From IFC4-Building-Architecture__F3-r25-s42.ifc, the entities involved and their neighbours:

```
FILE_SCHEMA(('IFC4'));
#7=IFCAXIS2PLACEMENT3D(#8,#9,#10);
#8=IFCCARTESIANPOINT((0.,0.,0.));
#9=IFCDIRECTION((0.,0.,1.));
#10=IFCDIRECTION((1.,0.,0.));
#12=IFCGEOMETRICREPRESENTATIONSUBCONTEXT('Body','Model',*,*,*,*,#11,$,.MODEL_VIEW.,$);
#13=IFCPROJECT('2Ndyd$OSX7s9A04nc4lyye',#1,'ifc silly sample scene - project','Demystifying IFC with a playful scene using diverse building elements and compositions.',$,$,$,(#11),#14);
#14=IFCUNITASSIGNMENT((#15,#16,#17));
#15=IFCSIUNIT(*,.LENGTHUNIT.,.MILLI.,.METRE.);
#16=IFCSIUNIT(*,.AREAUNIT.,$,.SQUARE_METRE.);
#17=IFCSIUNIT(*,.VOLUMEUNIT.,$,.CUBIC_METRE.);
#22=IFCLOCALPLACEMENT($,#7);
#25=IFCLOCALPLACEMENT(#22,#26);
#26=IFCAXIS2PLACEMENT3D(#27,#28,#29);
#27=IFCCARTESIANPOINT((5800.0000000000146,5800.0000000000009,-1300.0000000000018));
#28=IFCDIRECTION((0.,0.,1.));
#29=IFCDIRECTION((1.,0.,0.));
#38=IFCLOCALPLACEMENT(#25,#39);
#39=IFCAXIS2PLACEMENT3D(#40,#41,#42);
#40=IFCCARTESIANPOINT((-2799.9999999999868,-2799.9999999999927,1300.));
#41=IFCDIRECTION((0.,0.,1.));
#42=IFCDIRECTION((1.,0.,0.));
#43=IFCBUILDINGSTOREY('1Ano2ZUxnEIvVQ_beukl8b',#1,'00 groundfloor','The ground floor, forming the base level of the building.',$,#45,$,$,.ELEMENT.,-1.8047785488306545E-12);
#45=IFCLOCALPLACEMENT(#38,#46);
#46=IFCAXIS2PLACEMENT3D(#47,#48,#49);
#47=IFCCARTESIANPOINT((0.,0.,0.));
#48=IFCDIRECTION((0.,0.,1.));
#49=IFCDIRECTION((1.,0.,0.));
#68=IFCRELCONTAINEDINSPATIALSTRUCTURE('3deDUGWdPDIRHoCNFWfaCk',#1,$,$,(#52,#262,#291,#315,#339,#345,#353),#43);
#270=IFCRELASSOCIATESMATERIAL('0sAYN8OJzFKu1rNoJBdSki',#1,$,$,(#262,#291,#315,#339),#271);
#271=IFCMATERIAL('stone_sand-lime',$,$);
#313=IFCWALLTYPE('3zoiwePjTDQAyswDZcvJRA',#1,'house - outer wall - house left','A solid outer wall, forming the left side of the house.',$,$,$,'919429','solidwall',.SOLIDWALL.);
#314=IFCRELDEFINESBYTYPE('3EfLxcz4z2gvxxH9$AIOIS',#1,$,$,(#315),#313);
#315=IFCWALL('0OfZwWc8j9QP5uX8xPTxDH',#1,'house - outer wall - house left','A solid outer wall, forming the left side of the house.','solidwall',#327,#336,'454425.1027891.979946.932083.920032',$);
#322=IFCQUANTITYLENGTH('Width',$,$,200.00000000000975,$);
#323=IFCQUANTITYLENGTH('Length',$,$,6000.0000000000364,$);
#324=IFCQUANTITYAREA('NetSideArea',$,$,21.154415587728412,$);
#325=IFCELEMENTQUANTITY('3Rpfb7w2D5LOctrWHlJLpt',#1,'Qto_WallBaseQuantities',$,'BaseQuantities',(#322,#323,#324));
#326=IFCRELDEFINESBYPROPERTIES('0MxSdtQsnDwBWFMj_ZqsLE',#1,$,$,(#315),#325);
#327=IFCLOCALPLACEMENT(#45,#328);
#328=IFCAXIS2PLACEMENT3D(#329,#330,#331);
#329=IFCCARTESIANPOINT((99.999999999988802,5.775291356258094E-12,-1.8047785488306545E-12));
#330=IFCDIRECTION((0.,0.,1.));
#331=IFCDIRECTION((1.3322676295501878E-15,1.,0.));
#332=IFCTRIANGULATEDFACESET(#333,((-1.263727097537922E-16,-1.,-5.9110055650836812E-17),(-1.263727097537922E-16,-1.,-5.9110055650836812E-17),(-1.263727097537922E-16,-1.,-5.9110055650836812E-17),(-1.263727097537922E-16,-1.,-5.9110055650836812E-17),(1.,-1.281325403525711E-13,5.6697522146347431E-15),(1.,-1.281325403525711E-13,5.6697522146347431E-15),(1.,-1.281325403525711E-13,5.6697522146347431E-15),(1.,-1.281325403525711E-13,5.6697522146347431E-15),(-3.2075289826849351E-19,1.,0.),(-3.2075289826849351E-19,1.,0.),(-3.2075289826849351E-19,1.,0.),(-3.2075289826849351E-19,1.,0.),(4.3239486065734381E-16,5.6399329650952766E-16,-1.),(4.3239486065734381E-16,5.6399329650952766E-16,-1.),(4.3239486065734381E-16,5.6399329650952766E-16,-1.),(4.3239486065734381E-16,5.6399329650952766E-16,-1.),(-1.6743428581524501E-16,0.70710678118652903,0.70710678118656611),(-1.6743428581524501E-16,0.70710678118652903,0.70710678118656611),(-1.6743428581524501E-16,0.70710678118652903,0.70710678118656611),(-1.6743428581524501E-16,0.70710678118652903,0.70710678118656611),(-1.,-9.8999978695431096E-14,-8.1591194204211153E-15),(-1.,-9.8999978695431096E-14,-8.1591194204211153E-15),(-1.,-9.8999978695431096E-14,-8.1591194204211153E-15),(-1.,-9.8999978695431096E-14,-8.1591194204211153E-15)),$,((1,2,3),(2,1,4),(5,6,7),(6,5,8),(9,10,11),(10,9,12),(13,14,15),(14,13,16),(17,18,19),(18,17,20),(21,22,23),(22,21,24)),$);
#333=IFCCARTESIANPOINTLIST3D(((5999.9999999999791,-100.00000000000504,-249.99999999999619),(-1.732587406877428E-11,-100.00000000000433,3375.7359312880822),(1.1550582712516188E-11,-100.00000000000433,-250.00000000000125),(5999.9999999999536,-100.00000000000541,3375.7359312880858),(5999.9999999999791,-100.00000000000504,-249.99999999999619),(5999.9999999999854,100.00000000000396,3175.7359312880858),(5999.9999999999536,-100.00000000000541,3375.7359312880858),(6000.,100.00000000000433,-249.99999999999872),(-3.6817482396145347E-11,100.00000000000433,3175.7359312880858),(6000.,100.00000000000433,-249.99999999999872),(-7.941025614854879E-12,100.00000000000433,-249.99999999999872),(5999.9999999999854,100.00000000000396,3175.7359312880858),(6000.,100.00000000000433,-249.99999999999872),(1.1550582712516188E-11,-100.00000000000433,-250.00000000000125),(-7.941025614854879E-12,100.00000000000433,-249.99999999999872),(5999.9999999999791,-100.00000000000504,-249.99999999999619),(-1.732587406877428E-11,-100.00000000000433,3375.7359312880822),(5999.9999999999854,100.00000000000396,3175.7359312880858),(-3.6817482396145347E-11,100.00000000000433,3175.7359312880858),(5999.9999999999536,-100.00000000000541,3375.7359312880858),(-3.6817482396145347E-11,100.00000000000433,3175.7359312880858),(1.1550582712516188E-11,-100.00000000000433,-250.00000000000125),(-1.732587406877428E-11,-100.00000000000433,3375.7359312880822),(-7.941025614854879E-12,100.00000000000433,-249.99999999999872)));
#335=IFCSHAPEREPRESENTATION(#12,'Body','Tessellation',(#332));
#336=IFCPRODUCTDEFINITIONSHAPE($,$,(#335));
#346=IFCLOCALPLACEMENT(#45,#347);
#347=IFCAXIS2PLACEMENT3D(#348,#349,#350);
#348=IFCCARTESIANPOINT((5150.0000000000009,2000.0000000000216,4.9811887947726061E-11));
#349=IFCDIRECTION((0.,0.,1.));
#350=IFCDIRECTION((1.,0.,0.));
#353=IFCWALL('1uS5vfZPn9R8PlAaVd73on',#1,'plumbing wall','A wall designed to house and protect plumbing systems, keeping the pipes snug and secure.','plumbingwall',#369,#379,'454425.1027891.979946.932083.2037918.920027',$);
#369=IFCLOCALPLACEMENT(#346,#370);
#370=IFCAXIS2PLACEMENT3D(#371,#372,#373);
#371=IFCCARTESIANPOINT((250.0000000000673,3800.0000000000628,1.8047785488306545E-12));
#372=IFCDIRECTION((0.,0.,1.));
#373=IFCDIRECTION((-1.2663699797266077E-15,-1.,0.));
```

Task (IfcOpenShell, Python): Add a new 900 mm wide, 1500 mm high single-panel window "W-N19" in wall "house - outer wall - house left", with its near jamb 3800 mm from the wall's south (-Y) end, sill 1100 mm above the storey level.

```python
import numpy as np
import ifcopenshell
import ifcopenshell.api.feature
import ifcopenshell.api.geometry
import ifcopenshell.api.pset
import ifcopenshell.api.root
import ifcopenshell.api.spatial
import ifcopenshell.geom
import ifcopenshell.util.element
import ifcopenshell.util.placement
import ifcopenshell.util.representation
import ifcopenshell.util.shape
import ifcopenshell.util.unit

model = ifcopenshell.open("IFC4-Building-Architecture__F3-r25-s42.ifc")
unit_scale = ifcopenshell.util.unit.calculate_unit_scale(model)
area_scale = ifcopenshell.util.unit.calculate_unit_scale(model, "AREAUNIT")
settings = ifcopenshell.geom.settings()


def volume(element):
    """Net volume in cubic metres, openings subtracted."""
    shape = ifcopenshell.geom.create_shape(settings, element)
    return ifcopenshell.util.shape.get_volume(shape.geometry)


wall = model.by_guid("0OfZwWc8j9QP5uX8xPTxDH")
storey = ifcopenshell.util.element.get_container(wall, ifc_class="IfcBuildingStorey")
context = ifcopenshell.util.representation.get_context(model, "Model", "Body", "MODEL_VIEW")
before = volume(wall)

width, height, from_end, sill = 0.9, 1.5, 3.8, 1.1  # metres

# The wall runs along its own X axis, and the end named is its -X end.
wall_shape = ifcopenshell.geom.create_shape(settings, wall)
x, y, z = ifcopenshell.util.shape.get_vertices(wall_shape.geometry).T
start = x.min() + from_end
face, thickness = float(y.min()), float(y.max() - y.min())
wall_matrix = ifcopenshell.util.placement.get_local_placement(wall.ObjectPlacement)
level = ifcopenshell.util.placement.get_local_placement(storey.ObjectPlacement)[2, 3]


def in_wall(x, y):
    """Placement at x, y metres in the wall's axes, at sill height."""
    matrix = wall_matrix.copy()
    matrix[:, 3] = wall_matrix @ np.array([x / unit_scale, y / unit_scale, 0.0, 1.0])
    matrix[2, 3] = level + sill / unit_scale
    return matrix


# Opening: a box that overshoots both wall faces by 50 mm.
opening = ifcopenshell.api.root.create_entity(model, ifc_class="IfcOpeningElement", predefined_type="OPENING")
box = ifcopenshell.api.geometry.add_wall_representation(
    model, context=context, length=width, height=height, thickness=thickness + 0.1
)
ifcopenshell.api.geometry.assign_representation(model, product=opening, representation=box)
ifcopenshell.api.geometry.edit_object_placement(model, product=opening, matrix=in_wall(start, face - 0.05), is_si=False)
ifcopenshell.api.feature.add_feature(model, feature=opening, element=wall)

window = ifcopenshell.api.root.create_entity(model, ifc_class="IfcWindow", name="W-N19", predefined_type="WINDOW")
window.OverallWidth, window.OverallHeight = width / unit_scale, height / unit_scale
window.PartitioningType = "SINGLE_PANEL"
body = ifcopenshell.api.geometry.add_window_representation(
    model,
    context=context,
    overall_width=window.OverallWidth,
    overall_height=window.OverallHeight,
    partition_type="SINGLE_PANEL",
)
ifcopenshell.api.geometry.assign_representation(model, product=window, representation=body)
ifcopenshell.api.spatial.assign_container(model, products=[window], relating_structure=storey)
ifcopenshell.api.feature.add_filling(model, opening=opening, element=window)

# Centre the window in the wall's thickness.
ifcopenshell.api.geometry.edit_object_placement(model, product=window, matrix=in_wall(start, face), is_si=False)
window_shape = ifcopenshell.geom.create_shape(settings, window)
depth = ifcopenshell.util.shape.get_vertices(window_shape.geometry)[:, 1]
offset = face + thickness / 2 - (depth.min() + depth.max()) / 2
ifcopenshell.api.geometry.edit_object_placement(model, product=window, matrix=in_wall(start, offset), is_si=False)

after = volume(wall)

# Update the wall's stored quantities.
qto = model.by_id(ifcopenshell.util.element.get_pset(wall, "Qto_WallBaseQuantities", should_inherit=False)["id"])
ifcopenshell.api.pset.edit_qto(model, qto=qto, properties={"NetSideArea": after / thickness / area_scale})

print(f"wall volume {before:.3f} -> {after:.3f} m3")

model.write("IFC4-Building-Architecture__F3-r25-s42_v2.ifc")
```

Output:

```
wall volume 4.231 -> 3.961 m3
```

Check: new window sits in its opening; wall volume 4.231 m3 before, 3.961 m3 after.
